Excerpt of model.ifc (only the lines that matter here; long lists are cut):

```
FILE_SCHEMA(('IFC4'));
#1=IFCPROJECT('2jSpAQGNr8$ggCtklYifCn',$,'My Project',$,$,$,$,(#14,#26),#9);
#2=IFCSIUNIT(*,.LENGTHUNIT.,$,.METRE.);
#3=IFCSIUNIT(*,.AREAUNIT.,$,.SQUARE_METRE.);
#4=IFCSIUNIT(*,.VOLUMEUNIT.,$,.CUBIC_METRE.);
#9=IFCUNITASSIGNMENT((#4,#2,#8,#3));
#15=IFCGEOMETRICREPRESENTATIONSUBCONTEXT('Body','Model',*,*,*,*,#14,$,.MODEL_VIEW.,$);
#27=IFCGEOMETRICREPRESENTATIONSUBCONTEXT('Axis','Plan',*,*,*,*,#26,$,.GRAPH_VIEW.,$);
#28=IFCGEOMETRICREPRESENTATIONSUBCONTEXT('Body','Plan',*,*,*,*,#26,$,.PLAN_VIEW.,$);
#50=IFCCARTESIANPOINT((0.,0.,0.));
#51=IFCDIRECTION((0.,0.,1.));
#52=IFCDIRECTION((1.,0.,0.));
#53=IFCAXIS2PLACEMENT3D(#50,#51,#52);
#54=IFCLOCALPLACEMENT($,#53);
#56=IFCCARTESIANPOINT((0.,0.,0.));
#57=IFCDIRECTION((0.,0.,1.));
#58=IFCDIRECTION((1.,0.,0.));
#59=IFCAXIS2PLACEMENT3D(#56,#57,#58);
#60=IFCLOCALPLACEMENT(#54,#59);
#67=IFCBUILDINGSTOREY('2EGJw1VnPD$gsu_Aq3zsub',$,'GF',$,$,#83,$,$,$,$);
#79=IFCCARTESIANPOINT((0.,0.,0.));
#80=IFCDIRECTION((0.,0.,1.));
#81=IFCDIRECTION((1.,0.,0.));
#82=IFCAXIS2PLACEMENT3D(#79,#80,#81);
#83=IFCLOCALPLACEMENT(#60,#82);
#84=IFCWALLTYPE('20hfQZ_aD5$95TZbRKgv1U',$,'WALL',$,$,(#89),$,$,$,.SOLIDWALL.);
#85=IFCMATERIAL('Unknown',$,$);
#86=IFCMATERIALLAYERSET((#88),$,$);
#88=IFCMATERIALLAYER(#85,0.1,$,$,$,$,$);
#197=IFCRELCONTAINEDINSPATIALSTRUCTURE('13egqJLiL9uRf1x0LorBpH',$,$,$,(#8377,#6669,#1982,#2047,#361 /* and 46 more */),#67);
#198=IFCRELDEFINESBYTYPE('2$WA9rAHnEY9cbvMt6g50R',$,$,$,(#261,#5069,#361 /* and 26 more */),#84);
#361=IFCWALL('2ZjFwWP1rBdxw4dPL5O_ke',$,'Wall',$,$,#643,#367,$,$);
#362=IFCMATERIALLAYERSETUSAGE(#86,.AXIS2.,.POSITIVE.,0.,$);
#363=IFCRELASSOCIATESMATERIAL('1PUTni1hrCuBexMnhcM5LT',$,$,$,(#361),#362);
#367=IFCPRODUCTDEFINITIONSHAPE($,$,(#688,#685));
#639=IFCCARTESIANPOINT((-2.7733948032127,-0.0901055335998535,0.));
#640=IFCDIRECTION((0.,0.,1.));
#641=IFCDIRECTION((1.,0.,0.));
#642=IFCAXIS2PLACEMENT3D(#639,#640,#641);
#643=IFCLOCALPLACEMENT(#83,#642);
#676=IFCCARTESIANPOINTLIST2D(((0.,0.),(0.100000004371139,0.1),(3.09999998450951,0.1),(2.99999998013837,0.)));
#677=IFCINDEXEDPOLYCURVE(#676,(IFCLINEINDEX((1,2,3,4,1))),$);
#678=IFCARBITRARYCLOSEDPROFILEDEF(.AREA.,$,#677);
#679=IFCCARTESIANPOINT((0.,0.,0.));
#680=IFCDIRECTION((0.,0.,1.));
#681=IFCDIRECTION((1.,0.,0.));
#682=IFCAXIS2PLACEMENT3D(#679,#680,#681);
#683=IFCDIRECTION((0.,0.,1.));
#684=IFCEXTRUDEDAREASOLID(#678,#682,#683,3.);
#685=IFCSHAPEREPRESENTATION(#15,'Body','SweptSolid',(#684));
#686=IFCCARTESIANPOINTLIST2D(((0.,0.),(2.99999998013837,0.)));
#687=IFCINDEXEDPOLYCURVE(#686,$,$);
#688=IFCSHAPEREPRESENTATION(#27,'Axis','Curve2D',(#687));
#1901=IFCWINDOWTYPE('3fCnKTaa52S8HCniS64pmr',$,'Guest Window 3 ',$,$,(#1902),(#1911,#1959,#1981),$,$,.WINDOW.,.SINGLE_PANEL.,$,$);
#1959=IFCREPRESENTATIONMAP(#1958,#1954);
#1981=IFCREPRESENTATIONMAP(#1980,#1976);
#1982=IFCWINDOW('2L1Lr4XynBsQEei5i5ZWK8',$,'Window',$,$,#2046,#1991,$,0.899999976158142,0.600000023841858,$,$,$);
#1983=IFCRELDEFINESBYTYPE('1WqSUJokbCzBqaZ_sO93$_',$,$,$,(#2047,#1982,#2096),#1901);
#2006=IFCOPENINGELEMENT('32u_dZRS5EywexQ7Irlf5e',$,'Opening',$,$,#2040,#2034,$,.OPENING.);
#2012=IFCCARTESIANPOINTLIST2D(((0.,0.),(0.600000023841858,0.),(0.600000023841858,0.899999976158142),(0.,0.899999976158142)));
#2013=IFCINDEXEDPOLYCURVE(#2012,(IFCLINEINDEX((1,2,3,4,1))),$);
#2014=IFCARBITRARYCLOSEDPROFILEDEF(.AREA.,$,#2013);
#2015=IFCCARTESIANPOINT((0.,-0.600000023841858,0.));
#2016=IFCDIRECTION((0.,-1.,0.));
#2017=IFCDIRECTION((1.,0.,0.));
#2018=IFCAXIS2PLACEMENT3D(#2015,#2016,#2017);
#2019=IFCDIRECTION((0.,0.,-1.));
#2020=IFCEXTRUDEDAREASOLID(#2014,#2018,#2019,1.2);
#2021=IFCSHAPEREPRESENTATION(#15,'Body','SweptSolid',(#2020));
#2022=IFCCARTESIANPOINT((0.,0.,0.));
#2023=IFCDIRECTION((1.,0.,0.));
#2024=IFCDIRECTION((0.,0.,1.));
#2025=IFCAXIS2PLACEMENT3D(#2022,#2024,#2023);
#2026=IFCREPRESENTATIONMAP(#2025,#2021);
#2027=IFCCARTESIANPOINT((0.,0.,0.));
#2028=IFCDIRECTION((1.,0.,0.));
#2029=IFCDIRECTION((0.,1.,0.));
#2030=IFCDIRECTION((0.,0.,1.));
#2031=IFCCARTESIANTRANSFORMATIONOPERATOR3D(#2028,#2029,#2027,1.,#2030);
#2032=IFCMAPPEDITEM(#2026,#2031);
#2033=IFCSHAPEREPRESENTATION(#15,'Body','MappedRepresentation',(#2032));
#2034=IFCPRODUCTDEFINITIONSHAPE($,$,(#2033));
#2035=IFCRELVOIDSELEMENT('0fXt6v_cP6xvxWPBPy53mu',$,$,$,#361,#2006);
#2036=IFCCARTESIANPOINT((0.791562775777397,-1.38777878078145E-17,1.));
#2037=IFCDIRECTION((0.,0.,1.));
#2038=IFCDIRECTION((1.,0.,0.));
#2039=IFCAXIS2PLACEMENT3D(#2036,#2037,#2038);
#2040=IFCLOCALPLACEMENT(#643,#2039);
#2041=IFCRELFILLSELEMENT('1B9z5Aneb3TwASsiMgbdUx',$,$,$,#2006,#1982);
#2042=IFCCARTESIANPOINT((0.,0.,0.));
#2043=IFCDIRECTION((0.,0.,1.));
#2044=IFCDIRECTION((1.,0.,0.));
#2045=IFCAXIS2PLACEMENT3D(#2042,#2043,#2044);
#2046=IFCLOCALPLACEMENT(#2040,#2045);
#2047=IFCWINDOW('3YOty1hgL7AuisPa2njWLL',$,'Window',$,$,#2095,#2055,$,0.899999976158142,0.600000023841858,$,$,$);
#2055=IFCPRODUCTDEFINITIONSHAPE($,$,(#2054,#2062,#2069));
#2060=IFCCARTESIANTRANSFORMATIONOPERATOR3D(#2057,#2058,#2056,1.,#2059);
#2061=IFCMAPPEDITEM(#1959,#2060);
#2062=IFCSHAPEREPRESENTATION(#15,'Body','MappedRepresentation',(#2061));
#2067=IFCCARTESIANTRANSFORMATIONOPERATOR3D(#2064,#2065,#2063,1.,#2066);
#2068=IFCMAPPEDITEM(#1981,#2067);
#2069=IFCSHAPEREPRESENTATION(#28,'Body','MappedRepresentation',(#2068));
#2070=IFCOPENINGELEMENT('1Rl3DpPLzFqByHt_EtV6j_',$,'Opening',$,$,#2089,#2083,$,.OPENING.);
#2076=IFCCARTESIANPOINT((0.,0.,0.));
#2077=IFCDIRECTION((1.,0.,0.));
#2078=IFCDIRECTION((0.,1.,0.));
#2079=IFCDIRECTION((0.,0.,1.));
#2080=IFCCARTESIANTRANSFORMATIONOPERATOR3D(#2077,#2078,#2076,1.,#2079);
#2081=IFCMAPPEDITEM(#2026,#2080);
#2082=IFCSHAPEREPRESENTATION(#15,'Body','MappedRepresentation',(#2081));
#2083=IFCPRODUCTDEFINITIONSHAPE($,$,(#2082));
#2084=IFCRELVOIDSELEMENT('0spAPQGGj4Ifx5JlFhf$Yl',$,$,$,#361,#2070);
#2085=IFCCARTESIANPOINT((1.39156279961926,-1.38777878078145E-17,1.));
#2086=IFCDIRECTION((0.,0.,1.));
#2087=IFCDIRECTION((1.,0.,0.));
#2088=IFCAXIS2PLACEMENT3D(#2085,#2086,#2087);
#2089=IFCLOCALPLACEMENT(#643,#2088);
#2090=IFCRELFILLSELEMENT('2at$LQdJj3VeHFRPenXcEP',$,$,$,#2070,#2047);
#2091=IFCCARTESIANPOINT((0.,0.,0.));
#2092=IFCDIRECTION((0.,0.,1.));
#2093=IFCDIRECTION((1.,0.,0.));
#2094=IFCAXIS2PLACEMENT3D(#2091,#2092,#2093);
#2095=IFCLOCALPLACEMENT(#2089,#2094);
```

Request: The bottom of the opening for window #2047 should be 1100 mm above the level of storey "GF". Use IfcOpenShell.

```python
import numpy as np
import ifcopenshell
import ifcopenshell.api.geometry
import ifcopenshell.geom
import ifcopenshell.util.element
import ifcopenshell.util.placement
import ifcopenshell.util.shape
import ifcopenshell.util.unit

model = ifcopenshell.open("model.ifc")
unit_scale = ifcopenshell.util.unit.calculate_unit_scale(model)

window = model.by_guid("3YOty1hgL7AuisPa2njWLL")
opening = window.FillsVoids[0].RelatingOpeningElement
storey = ifcopenshell.util.element.get_container(window, ifc_class="IfcBuildingStorey")
level = ifcopenshell.util.placement.get_local_placement(storey.ObjectPlacement)[2, 3]

# The opening's origin need not be at the sill, so measure its lowest point.
shape = ifcopenshell.geom.create_shape(ifcopenshell.geom.settings(), opening)
bottom = ifcopenshell.util.shape.get_shape_bottom_elevation(shape, shape.geometry) / unit_scale
dz = level + 1.1 - bottom

shift = np.array([0.0, 0.0, dz])
# The window is placed relative to its opening, so it follows when the opening moves.
matrix = ifcopenshell.util.placement.get_local_placement(opening.ObjectPlacement)
matrix[:3, 3] += shift
ifcopenshell.api.geometry.edit_object_placement(
    model, product=opening, matrix=matrix, is_si=False, should_transform_children=True
)

print(f"moved by {dz * unit_scale:+.3f} m")

model.write("model_edited.ifc")
```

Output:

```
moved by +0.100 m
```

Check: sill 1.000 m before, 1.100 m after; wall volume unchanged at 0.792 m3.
